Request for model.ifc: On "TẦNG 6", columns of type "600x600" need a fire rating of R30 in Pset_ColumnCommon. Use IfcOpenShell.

First a look at what the model holds.

```python
import ifcopenshell
import ifcopenshell.util.element

model = ifcopenshell.open("model.ifc")
print(model.schema)
storey = next(s for s in model.by_type("IfcBuildingStorey") if s.Name == "TẦNG 6")
columns = [e for e in ifcopenshell.util.element.get_decomposition(storey) if e.is_a("IfcColumn")]
seen = {}
for e in columns:
    element_type = ifcopenshell.util.element.get_type(e)
    key = (element_type.Name if element_type != e and element_type else None, ifcopenshell.util.element.get_pset(e, "Pset_ColumnCommon", "FireRating"))
    seen[key] = seen.get(key, 0) + 1
for (name, value), count in sorted(seen.items(), key=str):
    print(count, "x", name, "|", value)
```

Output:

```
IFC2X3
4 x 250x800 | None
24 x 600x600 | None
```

```python
import ifcopenshell
import ifcopenshell.api.pset
import ifcopenshell.util.element

model = ifcopenshell.open("model.ifc")

storey = next(s for s in model.by_type("IfcBuildingStorey") if s.Name == "TẦNG 6")
columns = [e for e in ifcopenshell.util.element.get_decomposition(storey) if e.is_a("IfcColumn")]

count = 0
for e in columns:
    element_type = ifcopenshell.util.element.get_type(e)
    if element_type in (None, e) or element_type.Name != "600x600":
        continue
    # add_pset returns the element's existing set when there is one.
    pset = ifcopenshell.api.pset.add_pset(model, product=e, name="Pset_ColumnCommon")
    ifcopenshell.api.pset.edit_pset(model, pset=pset, properties={"FireRating": "R30"})
    count += 1

print(count, "columns updated")

model.write("model_v2.ifc")
```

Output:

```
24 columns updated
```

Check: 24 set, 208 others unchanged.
